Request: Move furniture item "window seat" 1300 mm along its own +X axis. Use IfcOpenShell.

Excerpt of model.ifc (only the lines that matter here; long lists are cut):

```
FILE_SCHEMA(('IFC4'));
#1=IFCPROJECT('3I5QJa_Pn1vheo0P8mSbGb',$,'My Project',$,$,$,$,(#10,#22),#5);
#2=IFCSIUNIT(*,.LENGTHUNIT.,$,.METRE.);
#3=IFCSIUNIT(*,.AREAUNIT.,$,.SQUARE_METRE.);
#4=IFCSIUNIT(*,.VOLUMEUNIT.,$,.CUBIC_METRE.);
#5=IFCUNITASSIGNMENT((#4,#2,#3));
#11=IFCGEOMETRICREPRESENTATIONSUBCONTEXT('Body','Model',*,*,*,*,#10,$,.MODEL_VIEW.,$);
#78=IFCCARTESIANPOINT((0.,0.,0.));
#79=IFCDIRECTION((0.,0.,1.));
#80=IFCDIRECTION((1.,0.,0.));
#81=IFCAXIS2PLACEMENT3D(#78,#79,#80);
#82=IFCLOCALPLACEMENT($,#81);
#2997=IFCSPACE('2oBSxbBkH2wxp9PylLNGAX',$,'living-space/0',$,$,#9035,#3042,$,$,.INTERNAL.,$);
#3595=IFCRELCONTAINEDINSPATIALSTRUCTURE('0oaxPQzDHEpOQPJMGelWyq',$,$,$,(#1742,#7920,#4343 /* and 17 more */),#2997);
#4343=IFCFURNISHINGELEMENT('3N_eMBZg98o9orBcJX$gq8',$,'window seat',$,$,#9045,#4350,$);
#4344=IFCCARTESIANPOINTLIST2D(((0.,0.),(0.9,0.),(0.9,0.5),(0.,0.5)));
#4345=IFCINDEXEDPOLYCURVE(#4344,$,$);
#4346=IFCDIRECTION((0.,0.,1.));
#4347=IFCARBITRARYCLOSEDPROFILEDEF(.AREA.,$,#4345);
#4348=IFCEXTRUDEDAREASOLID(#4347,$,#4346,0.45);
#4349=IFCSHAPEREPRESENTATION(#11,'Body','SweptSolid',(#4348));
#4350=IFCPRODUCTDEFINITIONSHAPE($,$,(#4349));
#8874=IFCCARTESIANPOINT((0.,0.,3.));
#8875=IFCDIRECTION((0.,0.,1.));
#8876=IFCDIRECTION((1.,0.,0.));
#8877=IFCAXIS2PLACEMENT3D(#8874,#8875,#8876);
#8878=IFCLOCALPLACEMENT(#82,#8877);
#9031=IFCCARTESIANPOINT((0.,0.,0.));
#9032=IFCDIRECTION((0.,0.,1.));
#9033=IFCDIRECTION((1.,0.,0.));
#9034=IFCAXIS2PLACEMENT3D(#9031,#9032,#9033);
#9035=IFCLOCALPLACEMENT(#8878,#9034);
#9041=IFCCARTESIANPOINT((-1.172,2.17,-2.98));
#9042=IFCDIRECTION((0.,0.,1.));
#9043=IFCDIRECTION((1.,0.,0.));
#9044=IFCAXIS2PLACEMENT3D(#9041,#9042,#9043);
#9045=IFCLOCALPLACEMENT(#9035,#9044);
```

```python
import ifcopenshell
import ifcopenshell.api.geometry
import ifcopenshell.util.placement

model = ifcopenshell.open("model.ifc")

item = model.by_guid("3N_eMBZg98o9orBcJX$gq8")
matrix = ifcopenshell.util.placement.get_local_placement(item.ObjectPlacement)
matrix[:3, 3] += matrix[:3, 0] * 1.3
ifcopenshell.api.geometry.edit_object_placement(model, product=item, matrix=matrix, is_si=False)

print(ifcopenshell.util.placement.get_local_placement(item.ObjectPlacement).round(3) + 0.0)

model.write("model_edited.ifc")
```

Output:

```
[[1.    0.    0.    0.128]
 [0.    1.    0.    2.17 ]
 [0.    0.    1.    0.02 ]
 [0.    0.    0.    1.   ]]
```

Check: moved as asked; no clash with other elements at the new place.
